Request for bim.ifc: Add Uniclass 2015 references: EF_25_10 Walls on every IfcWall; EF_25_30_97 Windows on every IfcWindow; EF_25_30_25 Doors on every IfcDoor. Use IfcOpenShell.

First a look at what the model holds.

```python
import ifcopenshell

model = ifcopenshell.open("bim.ifc")
print(model.schema)
print("classifications:", [c.Name for c in model.by_type("IfcClassification")])
for ifc_class in ("IfcDoor", "IfcRoof", "IfcStair", "IfcWall", "IfcWindow"):
    print(ifc_class, len(model.by_type(ifc_class)))
```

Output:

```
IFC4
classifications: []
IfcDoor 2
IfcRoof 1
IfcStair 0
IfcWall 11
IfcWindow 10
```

```python
import ifcopenshell
import ifcopenshell.api.classification

model = ifcopenshell.open("bim.ifc")

system = ifcopenshell.api.classification.add_classification(model, classification="Uniclass 2015")

codes = {
    "IfcWall": ("EF_25_10", "Walls"),
    "IfcWindow": ("EF_25_30_97", "Windows"),
    "IfcDoor": ("EF_25_30_25", "Doors"),
}
for ifc_class, (code, name) in codes.items():
    products = model.by_type(ifc_class)
    ifcopenshell.api.classification.add_reference(
        model, products=products, classification=system, identification=code, name=name
    )
    print(code, len(products))

model.write("bim_v2.ifc")
```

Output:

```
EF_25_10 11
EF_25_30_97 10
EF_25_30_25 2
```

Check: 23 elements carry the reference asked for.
